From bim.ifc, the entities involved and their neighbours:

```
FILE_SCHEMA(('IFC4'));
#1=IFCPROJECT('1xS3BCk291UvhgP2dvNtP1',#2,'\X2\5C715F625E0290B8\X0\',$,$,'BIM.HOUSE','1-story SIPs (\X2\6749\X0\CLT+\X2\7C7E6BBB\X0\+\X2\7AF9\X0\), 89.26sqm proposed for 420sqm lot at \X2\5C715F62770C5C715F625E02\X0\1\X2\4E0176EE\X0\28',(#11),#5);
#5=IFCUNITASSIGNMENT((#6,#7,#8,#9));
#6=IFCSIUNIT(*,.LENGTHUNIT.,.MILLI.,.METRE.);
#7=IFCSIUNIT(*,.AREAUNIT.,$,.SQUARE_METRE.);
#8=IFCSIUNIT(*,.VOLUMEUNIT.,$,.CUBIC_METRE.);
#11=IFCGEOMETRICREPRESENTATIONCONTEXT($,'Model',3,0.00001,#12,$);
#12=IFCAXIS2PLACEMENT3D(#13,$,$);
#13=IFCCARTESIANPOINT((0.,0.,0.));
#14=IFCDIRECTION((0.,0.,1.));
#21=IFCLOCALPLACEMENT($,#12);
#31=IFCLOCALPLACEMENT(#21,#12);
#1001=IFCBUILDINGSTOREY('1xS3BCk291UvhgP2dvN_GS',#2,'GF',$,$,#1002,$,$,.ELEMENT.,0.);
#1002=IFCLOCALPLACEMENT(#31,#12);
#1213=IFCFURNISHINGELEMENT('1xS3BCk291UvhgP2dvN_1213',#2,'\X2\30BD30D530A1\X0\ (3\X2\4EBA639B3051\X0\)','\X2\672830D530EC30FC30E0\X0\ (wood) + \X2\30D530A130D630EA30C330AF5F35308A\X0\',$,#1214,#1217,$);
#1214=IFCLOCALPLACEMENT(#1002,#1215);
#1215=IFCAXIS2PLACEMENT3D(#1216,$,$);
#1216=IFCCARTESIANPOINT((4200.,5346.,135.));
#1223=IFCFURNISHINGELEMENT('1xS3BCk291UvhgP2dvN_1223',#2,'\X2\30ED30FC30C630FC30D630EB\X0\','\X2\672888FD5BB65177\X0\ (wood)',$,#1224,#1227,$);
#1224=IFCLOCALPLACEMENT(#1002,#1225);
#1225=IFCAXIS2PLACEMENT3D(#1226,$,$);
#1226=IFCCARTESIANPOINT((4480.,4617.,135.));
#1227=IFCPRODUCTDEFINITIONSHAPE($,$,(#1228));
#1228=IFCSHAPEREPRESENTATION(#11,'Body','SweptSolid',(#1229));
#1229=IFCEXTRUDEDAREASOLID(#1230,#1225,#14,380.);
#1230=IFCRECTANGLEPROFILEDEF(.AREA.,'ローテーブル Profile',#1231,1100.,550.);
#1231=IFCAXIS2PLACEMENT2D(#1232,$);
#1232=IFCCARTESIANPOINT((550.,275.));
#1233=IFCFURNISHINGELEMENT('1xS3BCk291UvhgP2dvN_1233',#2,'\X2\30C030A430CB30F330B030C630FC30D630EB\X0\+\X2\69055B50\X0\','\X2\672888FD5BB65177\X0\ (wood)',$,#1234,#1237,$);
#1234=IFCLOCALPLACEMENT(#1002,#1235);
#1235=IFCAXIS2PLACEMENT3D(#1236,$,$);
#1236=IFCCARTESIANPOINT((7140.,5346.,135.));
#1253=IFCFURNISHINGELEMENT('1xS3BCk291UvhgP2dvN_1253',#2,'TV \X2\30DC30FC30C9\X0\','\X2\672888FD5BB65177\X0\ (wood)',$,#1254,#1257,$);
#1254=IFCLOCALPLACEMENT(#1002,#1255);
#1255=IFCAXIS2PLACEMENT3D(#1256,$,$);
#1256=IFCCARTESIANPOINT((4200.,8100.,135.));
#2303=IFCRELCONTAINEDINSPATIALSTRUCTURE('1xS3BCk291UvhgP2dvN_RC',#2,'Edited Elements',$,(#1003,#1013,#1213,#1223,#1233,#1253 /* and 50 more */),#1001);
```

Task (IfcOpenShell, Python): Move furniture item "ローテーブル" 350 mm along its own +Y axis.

```python
import ifcopenshell
import ifcopenshell.api.geometry
import ifcopenshell.util.placement

model = ifcopenshell.open("bim.ifc")

item = model.by_guid("1xS3BCk291UvhgP2dvN_1223")
matrix = ifcopenshell.util.placement.get_local_placement(item.ObjectPlacement)
matrix[:3, 3] += matrix[:3, 1] * 350.0
ifcopenshell.api.geometry.edit_object_placement(model, product=item, matrix=matrix, is_si=False)

print(ifcopenshell.util.placement.get_local_placement(item.ObjectPlacement).round(3) + 0.0)

model.write("bim_rev.ifc")
```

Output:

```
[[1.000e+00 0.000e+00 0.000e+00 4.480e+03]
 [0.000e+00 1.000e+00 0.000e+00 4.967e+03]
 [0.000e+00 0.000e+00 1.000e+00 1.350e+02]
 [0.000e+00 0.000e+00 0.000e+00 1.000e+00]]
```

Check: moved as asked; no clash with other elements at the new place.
